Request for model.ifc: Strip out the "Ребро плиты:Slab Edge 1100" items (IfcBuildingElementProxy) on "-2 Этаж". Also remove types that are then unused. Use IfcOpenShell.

First a look at what the model holds.

```python
import ifcopenshell
import ifcopenshell.util.element

model = ifcopenshell.open("model.ifc")
print(model.schema)
storey = next(s for s in model.by_type("IfcBuildingStorey") if s.Name == "-2 Этаж")
proxies = [e for e in ifcopenshell.util.element.get_decomposition(storey) if e.is_a("IfcBuildingElementProxy")]
seen = {}
for e in proxies:
    element_type = ifcopenshell.util.element.get_type(e)
    name = element_type.Name if element_type not in (None, e) else None
    seen[name] = seen.get(name, 0) + 1
for name, count in sorted(seen.items(), key=str):
    print(count, "x", name)
```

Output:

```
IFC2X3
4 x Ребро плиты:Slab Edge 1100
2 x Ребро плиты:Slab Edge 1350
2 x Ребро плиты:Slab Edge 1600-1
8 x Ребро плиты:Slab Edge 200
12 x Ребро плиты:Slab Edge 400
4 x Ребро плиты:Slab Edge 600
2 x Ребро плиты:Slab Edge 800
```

```python
import ifcopenshell
import ifcopenshell.api.root
import ifcopenshell.util.element

model = ifcopenshell.open("model.ifc")

storey = next(s for s in model.by_type("IfcBuildingStorey") if s.Name == "-2 Этаж")
proxies = [e for e in ifcopenshell.util.element.get_decomposition(storey) if e.is_a("IfcBuildingElementProxy")]
targets = [e for e in proxies if (t := ifcopenshell.util.element.get_type(e)) not in (None, e) and t.Name == "Ребро плиты:Slab Edge 1100"]
types = {ifcopenshell.util.element.get_type(e) for e in targets} - {None, *targets}

for e in targets:
    ifcopenshell.api.root.remove_product(model, product=e)
print(len(targets), "removed")

unused = [t for t in types if not ifcopenshell.util.element.get_types(t)]
for t in unused:
    ifcopenshell.api.root.remove_product(model, product=t)
print(len(unused), "unused types removed")

model.write("model-out.ifc")
```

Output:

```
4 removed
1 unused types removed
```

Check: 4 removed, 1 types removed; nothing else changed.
